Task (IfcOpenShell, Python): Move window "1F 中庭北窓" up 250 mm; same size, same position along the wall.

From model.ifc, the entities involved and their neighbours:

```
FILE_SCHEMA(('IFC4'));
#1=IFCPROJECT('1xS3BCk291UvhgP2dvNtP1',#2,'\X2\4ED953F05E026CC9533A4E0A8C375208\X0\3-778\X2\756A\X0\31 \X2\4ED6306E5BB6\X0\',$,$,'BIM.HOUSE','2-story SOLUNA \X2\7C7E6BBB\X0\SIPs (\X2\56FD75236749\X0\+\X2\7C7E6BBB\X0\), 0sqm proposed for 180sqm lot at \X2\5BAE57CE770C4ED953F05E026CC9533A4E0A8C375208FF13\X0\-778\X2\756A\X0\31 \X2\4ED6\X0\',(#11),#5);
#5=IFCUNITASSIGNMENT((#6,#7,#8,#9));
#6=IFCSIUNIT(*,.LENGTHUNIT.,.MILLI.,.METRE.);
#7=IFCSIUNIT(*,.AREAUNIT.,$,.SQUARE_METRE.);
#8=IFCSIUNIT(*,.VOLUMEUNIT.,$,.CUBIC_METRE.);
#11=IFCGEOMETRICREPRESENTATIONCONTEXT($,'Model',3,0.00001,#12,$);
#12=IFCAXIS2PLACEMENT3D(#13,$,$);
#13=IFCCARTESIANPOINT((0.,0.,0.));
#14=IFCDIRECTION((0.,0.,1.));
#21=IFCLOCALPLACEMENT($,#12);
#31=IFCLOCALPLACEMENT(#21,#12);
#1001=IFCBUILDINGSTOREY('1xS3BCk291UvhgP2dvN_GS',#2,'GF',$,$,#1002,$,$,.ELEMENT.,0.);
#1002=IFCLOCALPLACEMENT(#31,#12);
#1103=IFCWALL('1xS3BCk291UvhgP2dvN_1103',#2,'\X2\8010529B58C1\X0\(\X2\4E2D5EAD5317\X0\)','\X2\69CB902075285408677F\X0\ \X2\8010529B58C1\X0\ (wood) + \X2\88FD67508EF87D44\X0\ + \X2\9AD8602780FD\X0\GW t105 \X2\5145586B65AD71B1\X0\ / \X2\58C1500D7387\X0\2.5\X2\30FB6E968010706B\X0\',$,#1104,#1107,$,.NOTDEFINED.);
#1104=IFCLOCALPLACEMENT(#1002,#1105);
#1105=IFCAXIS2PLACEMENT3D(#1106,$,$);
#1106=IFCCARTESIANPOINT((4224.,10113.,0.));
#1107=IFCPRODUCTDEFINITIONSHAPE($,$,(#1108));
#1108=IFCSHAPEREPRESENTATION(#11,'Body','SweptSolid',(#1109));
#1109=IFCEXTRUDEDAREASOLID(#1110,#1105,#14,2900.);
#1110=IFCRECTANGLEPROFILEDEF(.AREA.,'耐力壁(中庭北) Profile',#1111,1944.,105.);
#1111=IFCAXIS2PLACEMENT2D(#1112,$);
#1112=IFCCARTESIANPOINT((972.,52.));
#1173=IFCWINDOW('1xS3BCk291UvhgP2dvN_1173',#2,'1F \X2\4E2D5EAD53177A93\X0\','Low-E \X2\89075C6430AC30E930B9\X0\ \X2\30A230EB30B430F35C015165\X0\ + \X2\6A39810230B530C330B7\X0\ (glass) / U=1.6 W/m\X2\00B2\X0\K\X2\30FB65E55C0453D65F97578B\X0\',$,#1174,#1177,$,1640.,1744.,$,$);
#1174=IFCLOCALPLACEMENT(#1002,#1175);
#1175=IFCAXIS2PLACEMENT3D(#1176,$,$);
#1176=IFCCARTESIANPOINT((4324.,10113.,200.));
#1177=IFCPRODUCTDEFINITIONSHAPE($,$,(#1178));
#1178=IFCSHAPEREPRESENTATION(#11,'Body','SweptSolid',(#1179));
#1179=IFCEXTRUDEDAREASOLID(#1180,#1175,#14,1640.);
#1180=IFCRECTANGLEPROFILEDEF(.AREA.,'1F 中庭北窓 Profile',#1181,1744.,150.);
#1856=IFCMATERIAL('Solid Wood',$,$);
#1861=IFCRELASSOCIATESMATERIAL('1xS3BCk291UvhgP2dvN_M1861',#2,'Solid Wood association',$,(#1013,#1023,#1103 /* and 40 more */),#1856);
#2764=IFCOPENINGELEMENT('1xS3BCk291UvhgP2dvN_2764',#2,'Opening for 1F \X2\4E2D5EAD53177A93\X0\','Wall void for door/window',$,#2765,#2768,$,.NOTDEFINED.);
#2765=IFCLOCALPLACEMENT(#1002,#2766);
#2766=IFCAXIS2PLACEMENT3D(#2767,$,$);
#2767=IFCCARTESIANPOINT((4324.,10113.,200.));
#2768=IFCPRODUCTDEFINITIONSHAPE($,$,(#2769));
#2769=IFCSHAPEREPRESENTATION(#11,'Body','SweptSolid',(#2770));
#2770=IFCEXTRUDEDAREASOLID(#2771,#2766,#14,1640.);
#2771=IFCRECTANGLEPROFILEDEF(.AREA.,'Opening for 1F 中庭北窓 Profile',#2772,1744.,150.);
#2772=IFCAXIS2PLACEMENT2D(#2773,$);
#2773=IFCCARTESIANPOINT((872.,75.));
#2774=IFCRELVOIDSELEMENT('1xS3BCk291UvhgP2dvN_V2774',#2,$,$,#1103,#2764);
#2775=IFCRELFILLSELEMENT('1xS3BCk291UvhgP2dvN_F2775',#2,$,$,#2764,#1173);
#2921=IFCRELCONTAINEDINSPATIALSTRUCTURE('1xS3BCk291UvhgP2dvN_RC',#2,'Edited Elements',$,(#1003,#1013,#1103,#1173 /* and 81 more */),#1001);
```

```python
import numpy as np
import ifcopenshell
import ifcopenshell.api.geometry
import ifcopenshell.util.placement
import ifcopenshell.util.unit

model = ifcopenshell.open("model.ifc")
unit_scale = ifcopenshell.util.unit.calculate_unit_scale(model)

window = model.by_guid("1xS3BCk291UvhgP2dvN_1173")
opening = window.FillsVoids[0].RelatingOpeningElement
dz = 250.0

shift = np.array([0.0, 0.0, dz])
# The window is not placed relative to its opening, so move both.
for product in (opening, window):
    matrix = ifcopenshell.util.placement.get_local_placement(product.ObjectPlacement)
    matrix[:3, 3] += shift
    ifcopenshell.api.geometry.edit_object_placement(model, product=product, matrix=matrix, is_si=False)

print(f"moved by {dz * unit_scale:+.3f} m")

model.write("model_edited.ifc")
```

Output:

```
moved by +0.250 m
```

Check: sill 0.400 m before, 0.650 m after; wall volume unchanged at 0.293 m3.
